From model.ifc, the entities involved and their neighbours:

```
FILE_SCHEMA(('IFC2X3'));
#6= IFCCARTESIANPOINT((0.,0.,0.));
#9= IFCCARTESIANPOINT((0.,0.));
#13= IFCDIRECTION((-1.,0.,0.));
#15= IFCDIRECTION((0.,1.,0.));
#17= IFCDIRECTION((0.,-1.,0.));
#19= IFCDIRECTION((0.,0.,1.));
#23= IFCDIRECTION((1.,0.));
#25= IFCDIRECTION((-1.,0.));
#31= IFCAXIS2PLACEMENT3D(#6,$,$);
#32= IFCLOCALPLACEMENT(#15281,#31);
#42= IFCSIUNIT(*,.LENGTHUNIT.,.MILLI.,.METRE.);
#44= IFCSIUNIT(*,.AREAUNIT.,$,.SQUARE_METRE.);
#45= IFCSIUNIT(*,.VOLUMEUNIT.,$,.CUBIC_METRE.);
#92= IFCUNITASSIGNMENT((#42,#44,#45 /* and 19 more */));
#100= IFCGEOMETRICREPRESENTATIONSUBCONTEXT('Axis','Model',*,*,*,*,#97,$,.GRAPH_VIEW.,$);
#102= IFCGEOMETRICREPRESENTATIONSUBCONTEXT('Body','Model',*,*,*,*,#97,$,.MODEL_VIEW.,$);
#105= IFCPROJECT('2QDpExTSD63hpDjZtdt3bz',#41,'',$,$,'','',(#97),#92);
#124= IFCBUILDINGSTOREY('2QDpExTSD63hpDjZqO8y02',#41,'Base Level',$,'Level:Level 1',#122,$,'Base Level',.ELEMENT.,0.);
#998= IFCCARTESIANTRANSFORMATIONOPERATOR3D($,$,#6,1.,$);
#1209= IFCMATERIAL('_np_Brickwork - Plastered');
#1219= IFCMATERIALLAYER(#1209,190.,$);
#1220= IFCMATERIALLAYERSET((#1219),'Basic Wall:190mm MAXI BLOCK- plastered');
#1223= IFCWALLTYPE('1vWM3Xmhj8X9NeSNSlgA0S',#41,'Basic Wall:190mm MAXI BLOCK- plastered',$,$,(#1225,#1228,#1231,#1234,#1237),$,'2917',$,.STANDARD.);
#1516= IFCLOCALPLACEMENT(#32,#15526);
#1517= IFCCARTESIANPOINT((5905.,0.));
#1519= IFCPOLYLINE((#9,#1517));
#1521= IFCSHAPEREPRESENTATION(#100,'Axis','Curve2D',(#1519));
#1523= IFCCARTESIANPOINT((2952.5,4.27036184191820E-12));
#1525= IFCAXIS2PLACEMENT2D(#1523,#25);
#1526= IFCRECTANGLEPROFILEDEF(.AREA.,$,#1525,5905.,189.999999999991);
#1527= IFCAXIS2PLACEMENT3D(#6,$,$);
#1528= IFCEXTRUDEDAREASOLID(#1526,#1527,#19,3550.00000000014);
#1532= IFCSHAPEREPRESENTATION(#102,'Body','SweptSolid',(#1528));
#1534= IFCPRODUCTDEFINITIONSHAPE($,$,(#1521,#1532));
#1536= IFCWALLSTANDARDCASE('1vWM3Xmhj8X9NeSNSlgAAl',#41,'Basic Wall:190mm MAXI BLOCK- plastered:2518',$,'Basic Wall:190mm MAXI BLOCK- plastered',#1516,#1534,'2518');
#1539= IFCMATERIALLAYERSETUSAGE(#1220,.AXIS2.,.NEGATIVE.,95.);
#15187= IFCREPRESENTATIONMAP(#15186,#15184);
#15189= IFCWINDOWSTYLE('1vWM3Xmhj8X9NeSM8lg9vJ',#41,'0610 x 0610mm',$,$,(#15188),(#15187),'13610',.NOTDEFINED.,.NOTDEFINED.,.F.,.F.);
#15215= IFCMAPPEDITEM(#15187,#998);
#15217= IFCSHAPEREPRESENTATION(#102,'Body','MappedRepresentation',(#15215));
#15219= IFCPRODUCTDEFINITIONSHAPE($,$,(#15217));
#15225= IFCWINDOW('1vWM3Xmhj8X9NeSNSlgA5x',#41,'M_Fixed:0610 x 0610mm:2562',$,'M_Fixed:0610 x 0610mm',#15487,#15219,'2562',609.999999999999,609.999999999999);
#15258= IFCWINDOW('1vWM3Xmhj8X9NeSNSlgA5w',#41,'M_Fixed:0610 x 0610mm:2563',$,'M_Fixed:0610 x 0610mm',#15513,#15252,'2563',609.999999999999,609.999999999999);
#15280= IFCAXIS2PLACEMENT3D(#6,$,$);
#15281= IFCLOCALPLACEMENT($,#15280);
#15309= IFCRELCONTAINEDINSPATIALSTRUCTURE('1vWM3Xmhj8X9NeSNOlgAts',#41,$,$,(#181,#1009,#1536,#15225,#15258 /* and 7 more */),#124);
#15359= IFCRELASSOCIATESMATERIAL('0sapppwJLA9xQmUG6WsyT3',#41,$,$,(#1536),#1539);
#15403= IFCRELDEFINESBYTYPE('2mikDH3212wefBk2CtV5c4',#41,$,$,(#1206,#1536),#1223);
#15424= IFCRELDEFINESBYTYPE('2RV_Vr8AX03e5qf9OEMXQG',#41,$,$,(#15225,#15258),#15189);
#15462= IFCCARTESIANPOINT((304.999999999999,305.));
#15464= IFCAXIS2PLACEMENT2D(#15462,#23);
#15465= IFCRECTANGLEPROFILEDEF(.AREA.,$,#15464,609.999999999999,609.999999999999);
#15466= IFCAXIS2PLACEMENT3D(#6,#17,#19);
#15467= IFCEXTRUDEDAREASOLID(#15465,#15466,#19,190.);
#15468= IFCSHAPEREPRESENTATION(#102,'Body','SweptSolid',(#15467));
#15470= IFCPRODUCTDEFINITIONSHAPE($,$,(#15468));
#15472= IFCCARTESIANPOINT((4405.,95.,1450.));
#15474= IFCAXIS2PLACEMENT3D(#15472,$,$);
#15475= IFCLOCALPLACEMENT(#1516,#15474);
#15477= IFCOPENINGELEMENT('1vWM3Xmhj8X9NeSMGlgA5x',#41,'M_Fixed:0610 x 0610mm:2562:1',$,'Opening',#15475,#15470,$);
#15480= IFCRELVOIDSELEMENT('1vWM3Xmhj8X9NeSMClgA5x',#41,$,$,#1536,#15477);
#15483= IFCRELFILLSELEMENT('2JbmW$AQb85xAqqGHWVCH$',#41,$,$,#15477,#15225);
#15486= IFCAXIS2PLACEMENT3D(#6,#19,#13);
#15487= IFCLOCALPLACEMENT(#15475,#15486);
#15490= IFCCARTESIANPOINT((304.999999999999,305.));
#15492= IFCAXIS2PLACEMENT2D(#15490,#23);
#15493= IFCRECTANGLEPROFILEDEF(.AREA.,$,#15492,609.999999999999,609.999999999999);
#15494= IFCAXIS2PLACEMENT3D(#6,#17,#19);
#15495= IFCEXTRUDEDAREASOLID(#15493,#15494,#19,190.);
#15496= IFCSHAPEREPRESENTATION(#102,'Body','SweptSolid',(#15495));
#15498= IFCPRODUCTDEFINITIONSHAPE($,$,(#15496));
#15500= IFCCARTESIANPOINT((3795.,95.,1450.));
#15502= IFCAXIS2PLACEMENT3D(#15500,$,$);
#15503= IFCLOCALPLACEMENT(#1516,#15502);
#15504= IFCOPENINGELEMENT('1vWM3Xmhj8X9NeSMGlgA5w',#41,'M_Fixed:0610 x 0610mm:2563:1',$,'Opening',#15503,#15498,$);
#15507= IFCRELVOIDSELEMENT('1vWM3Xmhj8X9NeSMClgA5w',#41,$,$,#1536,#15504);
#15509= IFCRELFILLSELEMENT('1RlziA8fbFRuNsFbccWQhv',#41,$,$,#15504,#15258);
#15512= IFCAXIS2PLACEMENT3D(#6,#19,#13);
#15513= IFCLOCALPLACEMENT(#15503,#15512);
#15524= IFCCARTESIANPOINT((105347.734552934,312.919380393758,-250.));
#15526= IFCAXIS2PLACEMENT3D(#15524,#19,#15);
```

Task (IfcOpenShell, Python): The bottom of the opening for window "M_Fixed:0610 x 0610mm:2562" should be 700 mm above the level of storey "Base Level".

```python
import numpy as np
import ifcopenshell
import ifcopenshell.api.geometry
import ifcopenshell.geom
import ifcopenshell.util.element
import ifcopenshell.util.placement
import ifcopenshell.util.shape
import ifcopenshell.util.unit

model = ifcopenshell.open("model.ifc")
unit_scale = ifcopenshell.util.unit.calculate_unit_scale(model)

window = model.by_guid("1vWM3Xmhj8X9NeSNSlgA5x")
opening = window.FillsVoids[0].RelatingOpeningElement
storey = ifcopenshell.util.element.get_container(window, ifc_class="IfcBuildingStorey")
level = ifcopenshell.util.placement.get_local_placement(storey.ObjectPlacement)[2, 3]

# The opening's origin need not be at the sill, so measure its lowest point.
shape = ifcopenshell.geom.create_shape(ifcopenshell.geom.settings(), opening)
bottom = ifcopenshell.util.shape.get_shape_bottom_elevation(shape, shape.geometry) / unit_scale
dz = level + 0.7 / unit_scale - bottom

shift = np.array([0.0, 0.0, dz])
# The window is placed relative to its opening, so it follows when the opening moves.
matrix = ifcopenshell.util.placement.get_local_placement(opening.ObjectPlacement)
matrix[:3, 3] += shift
ifcopenshell.api.geometry.edit_object_placement(
    model, product=opening, matrix=matrix, is_si=False, should_transform_children=True
)

print(f"moved by {dz * unit_scale:+.3f} m")

model.write("model-out.ifc")
```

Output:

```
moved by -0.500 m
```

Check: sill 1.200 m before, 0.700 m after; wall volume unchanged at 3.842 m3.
